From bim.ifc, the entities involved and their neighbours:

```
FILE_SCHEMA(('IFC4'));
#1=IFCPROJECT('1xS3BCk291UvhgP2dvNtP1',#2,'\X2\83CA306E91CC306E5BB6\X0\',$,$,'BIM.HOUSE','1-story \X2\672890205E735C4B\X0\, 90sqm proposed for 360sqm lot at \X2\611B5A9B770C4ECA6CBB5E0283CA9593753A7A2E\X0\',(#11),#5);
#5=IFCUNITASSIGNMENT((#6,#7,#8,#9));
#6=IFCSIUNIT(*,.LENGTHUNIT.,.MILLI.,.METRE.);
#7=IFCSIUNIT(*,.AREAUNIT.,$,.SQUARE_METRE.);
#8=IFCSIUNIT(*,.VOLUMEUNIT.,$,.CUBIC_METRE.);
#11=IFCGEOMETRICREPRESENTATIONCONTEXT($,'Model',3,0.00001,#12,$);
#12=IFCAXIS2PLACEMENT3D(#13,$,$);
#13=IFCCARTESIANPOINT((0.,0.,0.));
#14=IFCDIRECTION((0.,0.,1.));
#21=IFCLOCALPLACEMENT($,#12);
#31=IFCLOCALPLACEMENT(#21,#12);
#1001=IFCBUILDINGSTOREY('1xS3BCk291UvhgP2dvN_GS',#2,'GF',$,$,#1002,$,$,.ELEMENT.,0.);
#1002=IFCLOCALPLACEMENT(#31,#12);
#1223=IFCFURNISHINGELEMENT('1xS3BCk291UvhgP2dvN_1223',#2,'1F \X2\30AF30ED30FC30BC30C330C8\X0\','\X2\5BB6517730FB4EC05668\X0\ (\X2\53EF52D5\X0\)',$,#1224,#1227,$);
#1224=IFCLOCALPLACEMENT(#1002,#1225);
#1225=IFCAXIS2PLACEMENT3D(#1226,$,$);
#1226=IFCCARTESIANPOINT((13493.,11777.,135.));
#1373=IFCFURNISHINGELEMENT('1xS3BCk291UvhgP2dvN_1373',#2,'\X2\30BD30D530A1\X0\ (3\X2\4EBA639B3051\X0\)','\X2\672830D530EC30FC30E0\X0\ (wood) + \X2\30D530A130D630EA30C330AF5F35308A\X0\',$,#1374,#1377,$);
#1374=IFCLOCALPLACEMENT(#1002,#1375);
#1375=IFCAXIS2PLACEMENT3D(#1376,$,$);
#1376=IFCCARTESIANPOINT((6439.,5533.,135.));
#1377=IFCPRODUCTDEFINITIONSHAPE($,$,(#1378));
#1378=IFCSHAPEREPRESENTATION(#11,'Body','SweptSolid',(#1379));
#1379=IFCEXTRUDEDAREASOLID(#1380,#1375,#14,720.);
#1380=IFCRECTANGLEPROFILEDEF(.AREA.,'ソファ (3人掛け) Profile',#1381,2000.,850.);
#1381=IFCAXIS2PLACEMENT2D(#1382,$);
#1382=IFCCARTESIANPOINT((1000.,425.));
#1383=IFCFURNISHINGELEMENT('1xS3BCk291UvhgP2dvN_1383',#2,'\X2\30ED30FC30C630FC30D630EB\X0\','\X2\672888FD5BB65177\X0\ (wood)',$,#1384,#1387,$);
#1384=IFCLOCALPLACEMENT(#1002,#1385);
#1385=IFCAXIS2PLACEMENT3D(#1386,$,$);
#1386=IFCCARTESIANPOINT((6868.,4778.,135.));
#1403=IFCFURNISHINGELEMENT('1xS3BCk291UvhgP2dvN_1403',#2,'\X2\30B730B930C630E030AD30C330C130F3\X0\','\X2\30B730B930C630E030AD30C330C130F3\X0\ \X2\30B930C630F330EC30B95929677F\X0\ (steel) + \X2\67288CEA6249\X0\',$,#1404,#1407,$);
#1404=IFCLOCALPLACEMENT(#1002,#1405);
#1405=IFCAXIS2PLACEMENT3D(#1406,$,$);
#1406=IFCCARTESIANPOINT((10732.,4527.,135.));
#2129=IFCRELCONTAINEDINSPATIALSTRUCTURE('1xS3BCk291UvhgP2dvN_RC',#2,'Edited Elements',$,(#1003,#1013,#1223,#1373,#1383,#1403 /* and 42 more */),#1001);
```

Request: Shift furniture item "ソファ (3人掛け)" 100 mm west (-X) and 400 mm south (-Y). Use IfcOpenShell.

```python
import ifcopenshell
import ifcopenshell.api.geometry
import ifcopenshell.util.placement

model = ifcopenshell.open("bim.ifc")

item = model.by_guid("1xS3BCk291UvhgP2dvN_1373")
matrix = ifcopenshell.util.placement.get_local_placement(item.ObjectPlacement)
matrix[0, 3] -= 100.0
matrix[1, 3] -= 400.0
ifcopenshell.api.geometry.edit_object_placement(model, product=item, matrix=matrix, is_si=False)

print(ifcopenshell.util.placement.get_local_placement(item.ObjectPlacement).round(3) + 0.0)

model.write("bim_edited.ifc")
```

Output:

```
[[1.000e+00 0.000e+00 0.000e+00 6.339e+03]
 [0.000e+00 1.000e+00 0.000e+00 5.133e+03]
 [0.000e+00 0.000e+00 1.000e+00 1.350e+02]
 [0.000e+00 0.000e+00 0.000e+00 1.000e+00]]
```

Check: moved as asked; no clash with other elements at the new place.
